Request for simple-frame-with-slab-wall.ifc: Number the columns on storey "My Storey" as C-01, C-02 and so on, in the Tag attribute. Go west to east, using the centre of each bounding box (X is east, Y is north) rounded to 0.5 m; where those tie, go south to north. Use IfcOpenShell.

First a look at what the model holds.

```python
import ifcopenshell
import ifcopenshell.util.element
import ifcopenshell.util.placement

model = ifcopenshell.open("simple-frame-with-slab-wall.ifc")
print(model.schema)
storey = next(s for s in model.by_type("IfcBuildingStorey") if s.Name == "My Storey")
columns = [e for e in ifcopenshell.util.element.get_decomposition(storey) if e.is_a("IfcColumn")]
for e in sorted(columns, key=lambda e: e.id()):
    origin = ifcopenshell.util.placement.get_local_placement(e.ObjectPlacement)[:3, 3]
    print(e.id(), e.Tag, e.Name, origin.round(2) + 0.0, sep=" | ")
```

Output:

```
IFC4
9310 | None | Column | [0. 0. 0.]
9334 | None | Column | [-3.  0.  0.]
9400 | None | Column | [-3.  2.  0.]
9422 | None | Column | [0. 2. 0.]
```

```python
import ifcopenshell
import ifcopenshell.geom
import ifcopenshell.util.element
import ifcopenshell.util.shape

model = ifcopenshell.open("simple-frame-with-slab-wall.ifc")
settings = ifcopenshell.geom.settings()
settings.set("use-world-coords", True)


def centre(element):
    shape = ifcopenshell.geom.create_shape(settings, element)
    return ifcopenshell.util.shape.get_bbox_centroid(shape.geometry)


storey = next(s for s in model.by_type("IfcBuildingStorey") if s.Name == "My Storey")
columns = [e for e in ifcopenshell.util.element.get_decomposition(storey) if e.is_a("IfcColumn")]

# Insertion points can sit at a corner or the storey origin, so sort by the geometry (in metres).
centres = {e: centre(e) for e in columns}
columns.sort(key=lambda e: (round(centres[e][0] / 0.5), centres[e][1]))

for i, e in enumerate(columns, start=1):
    number = f"C-{i:02d}"
    e.Tag = number
    print(e.id(), number)

model.write("simple-frame-with-slab-wall_edited.ifc")
```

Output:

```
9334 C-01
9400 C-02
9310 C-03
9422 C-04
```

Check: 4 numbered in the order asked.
